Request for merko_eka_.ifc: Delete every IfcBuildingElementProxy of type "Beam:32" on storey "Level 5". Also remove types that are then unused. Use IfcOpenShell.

First a look at what the model holds.

```python
import ifcopenshell
import ifcopenshell.util.element

model = ifcopenshell.open("merko_eka_.ifc")
print(model.schema)
storey = next(s for s in model.by_type("IfcBuildingStorey") if s.Name == "Level 5")
proxies = [e for e in ifcopenshell.util.element.get_decomposition(storey) if e.is_a("IfcBuildingElementProxy")]
seen = {}
for e in proxies:
    element_type = ifcopenshell.util.element.get_type(e)
    name = element_type.Name if element_type not in (None, e) else None
    seen[name] = seen.get(name, 0) + 1
for name, count in sorted(seen.items(), key=str):
    print(count, "x", name)
```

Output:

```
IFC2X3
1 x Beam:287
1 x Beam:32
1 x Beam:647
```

```python
import ifcopenshell
import ifcopenshell.api.root
import ifcopenshell.util.element

model = ifcopenshell.open("merko_eka_.ifc")

storey = next(s for s in model.by_type("IfcBuildingStorey") if s.Name == "Level 5")
proxies = [e for e in ifcopenshell.util.element.get_decomposition(storey) if e.is_a("IfcBuildingElementProxy")]
targets = [e for e in proxies if (t := ifcopenshell.util.element.get_type(e)) not in (None, e) and t.Name == "Beam:32"]
types = {ifcopenshell.util.element.get_type(e) for e in targets} - {None, *targets}

for e in targets:
    ifcopenshell.api.root.remove_product(model, product=e)
print(len(targets), "removed")

unused = [t for t in types if not ifcopenshell.util.element.get_types(t)]
for t in unused:
    ifcopenshell.api.root.remove_product(model, product=t)
print(len(unused), "unused types removed")

model.write("merko_eka__v2.ifc")
```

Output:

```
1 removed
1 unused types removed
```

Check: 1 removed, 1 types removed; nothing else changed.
